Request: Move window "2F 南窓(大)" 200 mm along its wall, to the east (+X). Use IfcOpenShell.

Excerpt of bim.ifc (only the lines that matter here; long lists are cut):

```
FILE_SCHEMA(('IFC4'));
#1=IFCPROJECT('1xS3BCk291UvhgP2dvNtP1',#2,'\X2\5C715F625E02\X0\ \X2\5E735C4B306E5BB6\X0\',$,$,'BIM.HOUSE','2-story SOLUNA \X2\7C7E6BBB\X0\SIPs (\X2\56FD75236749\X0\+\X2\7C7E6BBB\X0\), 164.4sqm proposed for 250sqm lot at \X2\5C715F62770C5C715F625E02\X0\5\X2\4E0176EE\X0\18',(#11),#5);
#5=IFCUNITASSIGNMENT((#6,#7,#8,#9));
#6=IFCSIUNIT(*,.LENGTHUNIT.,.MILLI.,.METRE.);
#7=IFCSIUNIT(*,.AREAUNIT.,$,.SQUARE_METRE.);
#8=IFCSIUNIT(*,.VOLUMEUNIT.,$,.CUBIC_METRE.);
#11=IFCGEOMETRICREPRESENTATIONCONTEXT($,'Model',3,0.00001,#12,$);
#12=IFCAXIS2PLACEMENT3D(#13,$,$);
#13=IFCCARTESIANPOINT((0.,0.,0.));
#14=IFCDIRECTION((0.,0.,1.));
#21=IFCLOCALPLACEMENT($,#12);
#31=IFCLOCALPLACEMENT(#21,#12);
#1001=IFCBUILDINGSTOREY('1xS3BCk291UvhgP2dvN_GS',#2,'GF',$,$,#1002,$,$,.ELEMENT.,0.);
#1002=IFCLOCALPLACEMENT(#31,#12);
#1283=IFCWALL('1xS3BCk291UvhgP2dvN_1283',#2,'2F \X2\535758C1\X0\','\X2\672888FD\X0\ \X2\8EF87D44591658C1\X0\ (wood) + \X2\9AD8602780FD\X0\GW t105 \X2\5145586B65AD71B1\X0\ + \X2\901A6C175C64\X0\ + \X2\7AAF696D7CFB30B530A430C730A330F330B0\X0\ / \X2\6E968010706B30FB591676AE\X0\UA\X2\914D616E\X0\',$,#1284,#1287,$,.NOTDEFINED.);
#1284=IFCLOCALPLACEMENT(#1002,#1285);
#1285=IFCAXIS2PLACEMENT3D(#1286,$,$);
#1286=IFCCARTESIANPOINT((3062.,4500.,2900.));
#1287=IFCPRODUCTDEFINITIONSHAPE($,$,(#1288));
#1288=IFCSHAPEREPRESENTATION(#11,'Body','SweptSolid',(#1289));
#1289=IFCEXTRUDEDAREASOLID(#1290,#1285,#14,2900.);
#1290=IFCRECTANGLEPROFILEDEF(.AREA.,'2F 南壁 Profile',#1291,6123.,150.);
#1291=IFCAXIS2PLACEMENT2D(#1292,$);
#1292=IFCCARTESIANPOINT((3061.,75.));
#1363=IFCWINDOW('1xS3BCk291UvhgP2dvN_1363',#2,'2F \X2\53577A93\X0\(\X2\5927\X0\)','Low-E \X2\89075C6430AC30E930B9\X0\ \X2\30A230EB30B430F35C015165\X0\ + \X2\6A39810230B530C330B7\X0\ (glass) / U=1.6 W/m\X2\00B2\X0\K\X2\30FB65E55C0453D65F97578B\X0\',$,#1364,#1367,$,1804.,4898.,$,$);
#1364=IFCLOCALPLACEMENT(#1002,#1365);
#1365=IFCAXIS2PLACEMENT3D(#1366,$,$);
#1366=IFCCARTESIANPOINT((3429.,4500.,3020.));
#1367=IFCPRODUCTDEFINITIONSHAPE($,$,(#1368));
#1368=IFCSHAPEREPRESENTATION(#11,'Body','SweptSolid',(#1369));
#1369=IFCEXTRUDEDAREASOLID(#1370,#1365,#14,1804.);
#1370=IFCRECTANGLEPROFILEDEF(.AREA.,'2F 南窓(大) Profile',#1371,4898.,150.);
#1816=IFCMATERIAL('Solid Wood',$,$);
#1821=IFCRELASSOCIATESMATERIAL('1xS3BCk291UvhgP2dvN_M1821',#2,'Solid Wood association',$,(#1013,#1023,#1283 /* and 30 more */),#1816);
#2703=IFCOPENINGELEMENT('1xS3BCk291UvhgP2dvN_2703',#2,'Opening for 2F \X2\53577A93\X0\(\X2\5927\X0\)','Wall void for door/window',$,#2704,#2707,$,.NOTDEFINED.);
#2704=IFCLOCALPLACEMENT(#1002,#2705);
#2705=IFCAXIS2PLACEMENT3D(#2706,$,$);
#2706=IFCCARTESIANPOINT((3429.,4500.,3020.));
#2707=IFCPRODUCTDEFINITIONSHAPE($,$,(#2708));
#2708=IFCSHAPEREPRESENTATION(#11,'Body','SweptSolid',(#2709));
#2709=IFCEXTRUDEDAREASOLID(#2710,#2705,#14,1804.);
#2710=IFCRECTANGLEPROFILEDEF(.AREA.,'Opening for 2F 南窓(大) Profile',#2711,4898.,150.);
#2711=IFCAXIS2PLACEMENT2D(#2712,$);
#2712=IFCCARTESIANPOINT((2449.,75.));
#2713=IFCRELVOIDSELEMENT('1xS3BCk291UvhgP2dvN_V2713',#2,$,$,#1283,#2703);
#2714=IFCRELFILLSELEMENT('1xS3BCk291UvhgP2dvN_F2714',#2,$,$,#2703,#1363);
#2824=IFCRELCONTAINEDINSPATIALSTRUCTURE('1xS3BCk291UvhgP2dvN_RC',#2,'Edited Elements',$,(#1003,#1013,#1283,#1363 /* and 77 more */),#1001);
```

```python
import ifcopenshell
import ifcopenshell.api.geometry
import ifcopenshell.util.placement

model = ifcopenshell.open("bim.ifc")

window = model.by_id(1363)
opening = window.FillsVoids[0].RelatingOpeningElement
wall = opening.VoidsElements[0].RelatingBuildingElement

wall_matrix = ifcopenshell.util.placement.get_local_placement(wall.ObjectPlacement)
shift = wall_matrix[:3, 0] * 200.0
before = ifcopenshell.util.placement.get_local_placement(window.ObjectPlacement)[:3, 3].copy()

# The window is not placed relative to its opening, so move both.
for product in (opening, window):
    matrix = ifcopenshell.util.placement.get_local_placement(product.ObjectPlacement)
    matrix[:3, 3] += shift
    ifcopenshell.api.geometry.edit_object_placement(model, product=product, matrix=matrix, is_si=False)

after = ifcopenshell.util.placement.get_local_placement(window.ObjectPlacement)[:3, 3]
print("window moved by", (after - before).round(3) + 0.0)

model.write("bim-out.ifc")
```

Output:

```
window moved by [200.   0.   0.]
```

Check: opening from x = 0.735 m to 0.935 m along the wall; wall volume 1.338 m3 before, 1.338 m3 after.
